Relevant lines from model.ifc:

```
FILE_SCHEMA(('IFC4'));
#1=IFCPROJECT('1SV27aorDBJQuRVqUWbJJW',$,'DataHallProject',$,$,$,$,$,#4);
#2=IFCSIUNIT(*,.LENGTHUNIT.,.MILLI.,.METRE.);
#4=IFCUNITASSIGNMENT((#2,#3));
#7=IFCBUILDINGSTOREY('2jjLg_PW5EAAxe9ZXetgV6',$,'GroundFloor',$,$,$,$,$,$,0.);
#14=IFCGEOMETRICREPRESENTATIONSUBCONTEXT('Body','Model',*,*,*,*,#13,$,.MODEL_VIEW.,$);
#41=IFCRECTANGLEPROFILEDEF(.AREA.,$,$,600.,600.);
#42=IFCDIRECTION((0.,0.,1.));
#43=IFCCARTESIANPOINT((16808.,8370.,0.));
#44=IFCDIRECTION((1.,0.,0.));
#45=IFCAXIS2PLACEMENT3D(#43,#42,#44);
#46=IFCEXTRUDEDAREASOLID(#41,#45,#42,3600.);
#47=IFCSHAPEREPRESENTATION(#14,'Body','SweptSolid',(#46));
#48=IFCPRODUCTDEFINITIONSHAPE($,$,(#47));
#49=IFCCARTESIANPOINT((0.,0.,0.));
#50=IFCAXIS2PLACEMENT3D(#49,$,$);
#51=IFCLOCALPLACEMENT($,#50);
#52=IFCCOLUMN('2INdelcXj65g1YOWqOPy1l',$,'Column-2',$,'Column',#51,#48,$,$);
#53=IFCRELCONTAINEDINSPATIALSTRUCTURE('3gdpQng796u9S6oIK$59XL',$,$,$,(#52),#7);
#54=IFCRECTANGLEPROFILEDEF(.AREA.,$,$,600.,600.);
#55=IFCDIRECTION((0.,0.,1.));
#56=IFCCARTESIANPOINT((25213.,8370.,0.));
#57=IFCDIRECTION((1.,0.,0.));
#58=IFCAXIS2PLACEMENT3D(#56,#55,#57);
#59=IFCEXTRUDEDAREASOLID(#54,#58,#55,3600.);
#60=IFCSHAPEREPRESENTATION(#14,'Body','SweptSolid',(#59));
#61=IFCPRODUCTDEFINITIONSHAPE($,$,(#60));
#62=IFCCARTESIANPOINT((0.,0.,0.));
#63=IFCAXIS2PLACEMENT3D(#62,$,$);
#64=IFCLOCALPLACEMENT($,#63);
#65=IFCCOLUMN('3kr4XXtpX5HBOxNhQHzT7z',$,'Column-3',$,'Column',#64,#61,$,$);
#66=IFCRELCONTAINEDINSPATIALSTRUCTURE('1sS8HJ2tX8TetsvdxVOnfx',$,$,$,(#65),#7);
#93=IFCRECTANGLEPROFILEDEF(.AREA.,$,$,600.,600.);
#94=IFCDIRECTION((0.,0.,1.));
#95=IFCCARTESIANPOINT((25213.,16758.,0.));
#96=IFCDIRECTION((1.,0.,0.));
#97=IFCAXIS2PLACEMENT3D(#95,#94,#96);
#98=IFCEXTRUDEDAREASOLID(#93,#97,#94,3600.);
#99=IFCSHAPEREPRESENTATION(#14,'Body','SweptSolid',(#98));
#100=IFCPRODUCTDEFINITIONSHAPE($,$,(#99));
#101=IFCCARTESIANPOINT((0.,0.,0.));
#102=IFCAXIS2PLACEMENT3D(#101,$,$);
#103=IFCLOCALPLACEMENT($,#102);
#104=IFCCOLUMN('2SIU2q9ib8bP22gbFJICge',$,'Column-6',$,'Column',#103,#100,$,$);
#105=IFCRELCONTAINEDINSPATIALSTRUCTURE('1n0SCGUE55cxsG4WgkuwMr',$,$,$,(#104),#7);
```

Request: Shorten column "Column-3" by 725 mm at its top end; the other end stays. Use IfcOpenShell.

```python
import ifcopenshell
import ifcopenshell.util.representation

model = ifcopenshell.open("model.ifc")

member = model.by_id(65)
change = -725.0

# The extrusion runs towards the end named, so only its depth changes.
body = ifcopenshell.util.representation.get_representation(member, "Model", "Body")
solid = body.Items[0]
old_length = solid.Depth
solid.Depth += change

print(f"length {old_length:g} -> {solid.Depth:g}")

model.write("model-out.ifc")
```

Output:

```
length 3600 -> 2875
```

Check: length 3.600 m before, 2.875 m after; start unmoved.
